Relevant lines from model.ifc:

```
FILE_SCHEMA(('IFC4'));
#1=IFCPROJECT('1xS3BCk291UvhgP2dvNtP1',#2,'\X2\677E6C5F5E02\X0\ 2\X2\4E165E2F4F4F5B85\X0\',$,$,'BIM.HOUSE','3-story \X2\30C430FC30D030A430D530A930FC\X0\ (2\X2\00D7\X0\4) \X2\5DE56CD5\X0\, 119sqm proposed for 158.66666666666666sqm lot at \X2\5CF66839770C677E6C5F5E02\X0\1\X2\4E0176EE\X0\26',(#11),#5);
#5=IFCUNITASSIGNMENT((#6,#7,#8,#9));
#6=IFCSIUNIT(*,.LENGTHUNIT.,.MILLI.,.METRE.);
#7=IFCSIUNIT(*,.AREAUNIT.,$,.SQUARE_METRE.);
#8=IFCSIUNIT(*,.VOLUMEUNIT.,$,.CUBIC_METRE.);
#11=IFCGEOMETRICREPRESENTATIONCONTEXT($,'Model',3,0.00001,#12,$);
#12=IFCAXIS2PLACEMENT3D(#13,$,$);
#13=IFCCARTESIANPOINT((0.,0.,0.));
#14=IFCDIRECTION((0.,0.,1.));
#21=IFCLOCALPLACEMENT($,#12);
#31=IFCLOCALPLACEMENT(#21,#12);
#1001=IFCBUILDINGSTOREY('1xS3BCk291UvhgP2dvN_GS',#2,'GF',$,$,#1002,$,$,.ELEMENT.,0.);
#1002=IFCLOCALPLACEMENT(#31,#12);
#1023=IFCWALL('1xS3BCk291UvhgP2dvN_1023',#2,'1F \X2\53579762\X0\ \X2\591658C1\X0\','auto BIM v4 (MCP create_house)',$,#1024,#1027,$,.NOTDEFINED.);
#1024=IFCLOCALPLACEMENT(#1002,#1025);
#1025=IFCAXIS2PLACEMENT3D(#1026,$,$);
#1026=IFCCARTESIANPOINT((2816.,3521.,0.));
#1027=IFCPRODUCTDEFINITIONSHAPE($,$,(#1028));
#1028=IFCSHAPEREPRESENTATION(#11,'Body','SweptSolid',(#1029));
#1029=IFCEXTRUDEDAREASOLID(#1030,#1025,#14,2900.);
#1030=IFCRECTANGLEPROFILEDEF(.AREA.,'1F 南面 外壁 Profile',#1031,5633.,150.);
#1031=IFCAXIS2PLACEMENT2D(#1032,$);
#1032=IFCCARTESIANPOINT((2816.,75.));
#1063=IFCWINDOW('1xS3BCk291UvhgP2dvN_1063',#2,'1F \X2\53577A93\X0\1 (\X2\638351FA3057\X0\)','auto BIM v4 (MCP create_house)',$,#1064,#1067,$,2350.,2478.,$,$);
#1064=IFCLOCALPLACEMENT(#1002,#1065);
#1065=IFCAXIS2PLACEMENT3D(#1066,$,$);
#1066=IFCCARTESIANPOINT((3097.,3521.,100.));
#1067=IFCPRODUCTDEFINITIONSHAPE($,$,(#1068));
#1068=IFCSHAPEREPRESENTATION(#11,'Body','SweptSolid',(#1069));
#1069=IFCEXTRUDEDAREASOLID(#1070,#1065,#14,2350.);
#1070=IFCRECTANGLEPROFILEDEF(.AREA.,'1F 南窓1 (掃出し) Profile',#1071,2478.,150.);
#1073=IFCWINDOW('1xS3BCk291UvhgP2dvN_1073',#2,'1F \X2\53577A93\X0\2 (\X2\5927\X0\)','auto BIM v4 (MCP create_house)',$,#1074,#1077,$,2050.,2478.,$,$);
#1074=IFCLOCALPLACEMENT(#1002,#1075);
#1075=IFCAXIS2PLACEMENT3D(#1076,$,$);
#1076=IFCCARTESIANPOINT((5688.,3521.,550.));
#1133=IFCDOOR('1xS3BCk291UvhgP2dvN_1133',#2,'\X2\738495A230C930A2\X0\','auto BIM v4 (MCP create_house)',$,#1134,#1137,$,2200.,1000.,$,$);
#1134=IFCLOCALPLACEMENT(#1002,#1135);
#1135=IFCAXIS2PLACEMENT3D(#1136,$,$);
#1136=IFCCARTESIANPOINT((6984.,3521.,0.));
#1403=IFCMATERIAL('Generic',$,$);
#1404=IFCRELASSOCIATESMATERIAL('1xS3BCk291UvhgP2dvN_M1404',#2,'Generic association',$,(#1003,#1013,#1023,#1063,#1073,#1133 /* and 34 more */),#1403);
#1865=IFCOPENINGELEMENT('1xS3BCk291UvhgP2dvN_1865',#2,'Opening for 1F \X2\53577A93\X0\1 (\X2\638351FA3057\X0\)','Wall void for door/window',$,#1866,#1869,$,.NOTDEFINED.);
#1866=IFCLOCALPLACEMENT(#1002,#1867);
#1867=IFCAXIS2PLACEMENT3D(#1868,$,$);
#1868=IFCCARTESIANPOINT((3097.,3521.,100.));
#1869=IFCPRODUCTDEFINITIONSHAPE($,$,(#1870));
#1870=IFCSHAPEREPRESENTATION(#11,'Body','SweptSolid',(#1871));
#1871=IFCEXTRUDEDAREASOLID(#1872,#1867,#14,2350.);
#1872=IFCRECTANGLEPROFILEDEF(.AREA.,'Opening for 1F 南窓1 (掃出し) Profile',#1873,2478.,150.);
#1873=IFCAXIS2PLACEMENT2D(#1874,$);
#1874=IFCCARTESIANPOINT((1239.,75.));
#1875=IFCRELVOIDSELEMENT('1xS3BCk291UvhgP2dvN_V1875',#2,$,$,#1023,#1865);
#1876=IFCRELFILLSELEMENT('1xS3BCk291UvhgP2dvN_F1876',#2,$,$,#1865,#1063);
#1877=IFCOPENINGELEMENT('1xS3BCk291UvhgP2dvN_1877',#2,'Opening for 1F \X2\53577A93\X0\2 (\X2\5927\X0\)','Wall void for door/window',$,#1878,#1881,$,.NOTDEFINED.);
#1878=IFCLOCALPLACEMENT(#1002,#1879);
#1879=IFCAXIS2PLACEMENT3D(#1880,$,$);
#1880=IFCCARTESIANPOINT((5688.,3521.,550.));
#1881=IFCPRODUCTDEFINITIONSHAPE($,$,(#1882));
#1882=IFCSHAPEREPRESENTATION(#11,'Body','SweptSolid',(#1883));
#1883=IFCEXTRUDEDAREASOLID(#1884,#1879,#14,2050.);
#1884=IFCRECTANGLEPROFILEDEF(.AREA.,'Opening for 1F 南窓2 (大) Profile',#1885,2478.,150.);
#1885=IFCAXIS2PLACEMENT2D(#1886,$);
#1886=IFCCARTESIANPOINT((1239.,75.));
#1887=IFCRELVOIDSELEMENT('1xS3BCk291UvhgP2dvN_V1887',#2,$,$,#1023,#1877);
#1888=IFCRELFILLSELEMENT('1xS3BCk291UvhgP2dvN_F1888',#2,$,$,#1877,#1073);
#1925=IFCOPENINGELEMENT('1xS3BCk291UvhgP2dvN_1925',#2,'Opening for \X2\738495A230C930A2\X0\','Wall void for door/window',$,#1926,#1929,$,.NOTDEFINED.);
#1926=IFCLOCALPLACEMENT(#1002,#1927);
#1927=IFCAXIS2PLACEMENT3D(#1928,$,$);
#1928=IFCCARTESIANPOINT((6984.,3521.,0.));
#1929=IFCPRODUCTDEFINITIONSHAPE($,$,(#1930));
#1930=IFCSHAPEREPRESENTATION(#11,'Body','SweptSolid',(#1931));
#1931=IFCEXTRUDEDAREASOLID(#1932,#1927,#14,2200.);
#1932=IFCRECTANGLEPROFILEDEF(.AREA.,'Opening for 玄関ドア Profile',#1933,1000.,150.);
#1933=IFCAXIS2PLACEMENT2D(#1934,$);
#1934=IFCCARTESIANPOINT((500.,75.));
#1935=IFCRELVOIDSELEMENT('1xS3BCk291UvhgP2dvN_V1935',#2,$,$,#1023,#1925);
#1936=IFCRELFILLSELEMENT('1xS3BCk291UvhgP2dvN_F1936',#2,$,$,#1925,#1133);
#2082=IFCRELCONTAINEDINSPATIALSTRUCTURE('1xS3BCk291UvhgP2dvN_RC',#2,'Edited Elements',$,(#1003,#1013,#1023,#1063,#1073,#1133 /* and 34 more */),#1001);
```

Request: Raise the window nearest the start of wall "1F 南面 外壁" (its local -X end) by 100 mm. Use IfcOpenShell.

```python
import numpy as np
import ifcopenshell
import ifcopenshell.api.geometry
import ifcopenshell.util.placement
import ifcopenshell.util.unit

model = ifcopenshell.open("model.ifc")
unit_scale = ifcopenshell.util.unit.calculate_unit_scale(model)

window = model.by_guid("1xS3BCk291UvhgP2dvN_1063")
opening = window.FillsVoids[0].RelatingOpeningElement
dz = 100.0

shift = np.array([0.0, 0.0, dz])
# The window is not placed relative to its opening, so move both.
for product in (opening, window):
    matrix = ifcopenshell.util.placement.get_local_placement(product.ObjectPlacement)
    matrix[:3, 3] += shift
    ifcopenshell.api.geometry.edit_object_placement(model, product=product, matrix=matrix, is_si=False)

print(f"moved by {dz * unit_scale:+.3f} m")

model.write("model_v2.ifc")
```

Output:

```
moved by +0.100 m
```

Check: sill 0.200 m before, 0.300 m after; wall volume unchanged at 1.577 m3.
